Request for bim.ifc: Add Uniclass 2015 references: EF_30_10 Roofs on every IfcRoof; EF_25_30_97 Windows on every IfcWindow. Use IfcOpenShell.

First a look at what the model holds.

```python
import ifcopenshell

model = ifcopenshell.open("bim.ifc")
print(model.schema)
print("classifications:", [c.Name for c in model.by_type("IfcClassification")])
for ifc_class in ("IfcDoor", "IfcRoof", "IfcStair", "IfcWall", "IfcWindow"):
    print(ifc_class, len(model.by_type(ifc_class)))
```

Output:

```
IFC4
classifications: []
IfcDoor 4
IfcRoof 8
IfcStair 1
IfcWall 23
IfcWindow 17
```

```python
import ifcopenshell
import ifcopenshell.api.classification

model = ifcopenshell.open("bim.ifc")

system = ifcopenshell.api.classification.add_classification(model, classification="Uniclass 2015")

codes = {
    "IfcRoof": ("EF_30_10", "Roofs"),
    "IfcWindow": ("EF_25_30_97", "Windows"),
}
for ifc_class, (code, name) in codes.items():
    products = model.by_type(ifc_class)
    ifcopenshell.api.classification.add_reference(
        model, products=products, classification=system, identification=code, name=name
    )
    print(code, len(products))

model.write("bim_v2.ifc")
```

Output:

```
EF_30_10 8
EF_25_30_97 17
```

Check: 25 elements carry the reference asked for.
